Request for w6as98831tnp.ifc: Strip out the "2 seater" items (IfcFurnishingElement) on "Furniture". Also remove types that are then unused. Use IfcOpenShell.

First a look at what the model holds.

```python
import ifcopenshell
import ifcopenshell.util.element

model = ifcopenshell.open("w6as98831tnp.ifc")
print(model.schema)
storey = next(s for s in model.by_type("IfcBuildingStorey") if s.Name == "Furniture")
furniture = [e for e in ifcopenshell.util.element.get_decomposition(storey) if e.is_a("IfcFurnishingElement")]
seen = {}
for e in furniture:
    element_type = ifcopenshell.util.element.get_type(e)
    name = element_type.Name if element_type not in (None, e) else None
    seen[name] = seen.get(name, 0) + 1
for name, count in sorted(seen.items(), key=str):
    print(count, "x", name)
```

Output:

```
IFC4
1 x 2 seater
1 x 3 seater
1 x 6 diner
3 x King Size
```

```python
import ifcopenshell
import ifcopenshell.api.root
import ifcopenshell.util.element

model = ifcopenshell.open("w6as98831tnp.ifc")

storey = next(s for s in model.by_type("IfcBuildingStorey") if s.Name == "Furniture")
furniture = [e for e in ifcopenshell.util.element.get_decomposition(storey) if e.is_a("IfcFurnishingElement")]
targets = [e for e in furniture if (t := ifcopenshell.util.element.get_type(e)) not in (None, e) and t.Name == "2 seater"]
types = {ifcopenshell.util.element.get_type(e) for e in targets} - {None, *targets}

for e in targets:
    ifcopenshell.api.root.remove_product(model, product=e)
print(len(targets), "removed")

unused = [t for t in types if not ifcopenshell.util.element.get_types(t)]
for t in unused:
    ifcopenshell.api.root.remove_product(model, product=t)
print(len(unused), "unused types removed")

model.write("w6as98831tnp_edited.ifc")
```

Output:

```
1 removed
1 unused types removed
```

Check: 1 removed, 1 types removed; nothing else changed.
